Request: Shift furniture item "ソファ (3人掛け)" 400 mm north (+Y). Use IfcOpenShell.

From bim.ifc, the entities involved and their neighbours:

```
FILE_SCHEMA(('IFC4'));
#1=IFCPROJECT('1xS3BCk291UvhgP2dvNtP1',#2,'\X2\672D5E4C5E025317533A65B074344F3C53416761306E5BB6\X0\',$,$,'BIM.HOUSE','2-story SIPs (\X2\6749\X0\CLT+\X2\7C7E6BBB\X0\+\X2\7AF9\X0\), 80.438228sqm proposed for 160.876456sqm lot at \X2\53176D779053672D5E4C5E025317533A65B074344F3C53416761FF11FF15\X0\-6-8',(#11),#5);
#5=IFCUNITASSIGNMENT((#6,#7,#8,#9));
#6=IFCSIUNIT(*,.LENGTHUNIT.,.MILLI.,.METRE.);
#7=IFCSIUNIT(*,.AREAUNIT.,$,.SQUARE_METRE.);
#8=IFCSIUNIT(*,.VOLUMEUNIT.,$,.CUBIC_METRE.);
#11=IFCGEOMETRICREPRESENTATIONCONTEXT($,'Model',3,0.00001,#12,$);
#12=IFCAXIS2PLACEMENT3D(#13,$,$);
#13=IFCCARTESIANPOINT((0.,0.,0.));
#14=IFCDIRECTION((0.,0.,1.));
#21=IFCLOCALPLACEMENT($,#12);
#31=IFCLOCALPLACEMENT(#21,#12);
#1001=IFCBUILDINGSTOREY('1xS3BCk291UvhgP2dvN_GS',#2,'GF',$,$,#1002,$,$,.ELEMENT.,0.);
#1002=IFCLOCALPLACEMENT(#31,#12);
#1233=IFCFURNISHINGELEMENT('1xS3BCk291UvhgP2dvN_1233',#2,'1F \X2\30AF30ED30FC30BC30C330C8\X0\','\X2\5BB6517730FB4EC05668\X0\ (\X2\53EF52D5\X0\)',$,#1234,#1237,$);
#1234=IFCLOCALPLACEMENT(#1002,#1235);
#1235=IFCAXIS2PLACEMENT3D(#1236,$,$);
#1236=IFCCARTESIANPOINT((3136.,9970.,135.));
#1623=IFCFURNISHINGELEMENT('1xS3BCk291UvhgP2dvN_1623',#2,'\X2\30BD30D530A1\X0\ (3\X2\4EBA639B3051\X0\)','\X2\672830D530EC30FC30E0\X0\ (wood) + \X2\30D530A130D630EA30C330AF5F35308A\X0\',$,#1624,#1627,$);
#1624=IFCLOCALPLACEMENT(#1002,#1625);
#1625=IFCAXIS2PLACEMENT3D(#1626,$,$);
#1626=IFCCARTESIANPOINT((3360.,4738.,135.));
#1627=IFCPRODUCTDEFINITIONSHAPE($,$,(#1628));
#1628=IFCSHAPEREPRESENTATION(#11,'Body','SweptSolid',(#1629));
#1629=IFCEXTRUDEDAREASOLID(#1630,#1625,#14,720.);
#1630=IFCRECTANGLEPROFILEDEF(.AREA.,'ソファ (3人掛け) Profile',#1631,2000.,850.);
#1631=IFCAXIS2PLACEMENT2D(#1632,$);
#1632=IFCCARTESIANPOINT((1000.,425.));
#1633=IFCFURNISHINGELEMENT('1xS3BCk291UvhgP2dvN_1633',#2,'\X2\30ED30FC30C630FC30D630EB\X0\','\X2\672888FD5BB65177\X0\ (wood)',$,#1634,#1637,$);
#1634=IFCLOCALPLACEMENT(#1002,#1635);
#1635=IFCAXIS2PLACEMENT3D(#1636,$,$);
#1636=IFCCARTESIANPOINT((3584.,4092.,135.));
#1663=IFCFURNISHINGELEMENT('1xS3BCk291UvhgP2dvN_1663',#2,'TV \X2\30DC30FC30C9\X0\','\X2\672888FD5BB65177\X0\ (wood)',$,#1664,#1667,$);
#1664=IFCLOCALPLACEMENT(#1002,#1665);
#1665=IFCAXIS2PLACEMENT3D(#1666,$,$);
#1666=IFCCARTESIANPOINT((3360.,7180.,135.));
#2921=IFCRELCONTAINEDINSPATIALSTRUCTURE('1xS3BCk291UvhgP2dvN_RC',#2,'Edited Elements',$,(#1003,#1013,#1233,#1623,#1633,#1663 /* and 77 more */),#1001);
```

```python
import ifcopenshell
import ifcopenshell.api.geometry
import ifcopenshell.util.placement
import ifcopenshell.util.unit

model = ifcopenshell.open("bim.ifc")
unit_scale = ifcopenshell.util.unit.calculate_unit_scale(model)

item = model.by_guid("1xS3BCk291UvhgP2dvN_1623")
matrix = ifcopenshell.util.placement.get_local_placement(item.ObjectPlacement)
matrix[1, 3] += 0.4 / unit_scale
ifcopenshell.api.geometry.edit_object_placement(model, product=item, matrix=matrix, is_si=False)

print(ifcopenshell.util.placement.get_local_placement(item.ObjectPlacement).round(3) + 0.0)

model.write("bim_updated.ifc")
```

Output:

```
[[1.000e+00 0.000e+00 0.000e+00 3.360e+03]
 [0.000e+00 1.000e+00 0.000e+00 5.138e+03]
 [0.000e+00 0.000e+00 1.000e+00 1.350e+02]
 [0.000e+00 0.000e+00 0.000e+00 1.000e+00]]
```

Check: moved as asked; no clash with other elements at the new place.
